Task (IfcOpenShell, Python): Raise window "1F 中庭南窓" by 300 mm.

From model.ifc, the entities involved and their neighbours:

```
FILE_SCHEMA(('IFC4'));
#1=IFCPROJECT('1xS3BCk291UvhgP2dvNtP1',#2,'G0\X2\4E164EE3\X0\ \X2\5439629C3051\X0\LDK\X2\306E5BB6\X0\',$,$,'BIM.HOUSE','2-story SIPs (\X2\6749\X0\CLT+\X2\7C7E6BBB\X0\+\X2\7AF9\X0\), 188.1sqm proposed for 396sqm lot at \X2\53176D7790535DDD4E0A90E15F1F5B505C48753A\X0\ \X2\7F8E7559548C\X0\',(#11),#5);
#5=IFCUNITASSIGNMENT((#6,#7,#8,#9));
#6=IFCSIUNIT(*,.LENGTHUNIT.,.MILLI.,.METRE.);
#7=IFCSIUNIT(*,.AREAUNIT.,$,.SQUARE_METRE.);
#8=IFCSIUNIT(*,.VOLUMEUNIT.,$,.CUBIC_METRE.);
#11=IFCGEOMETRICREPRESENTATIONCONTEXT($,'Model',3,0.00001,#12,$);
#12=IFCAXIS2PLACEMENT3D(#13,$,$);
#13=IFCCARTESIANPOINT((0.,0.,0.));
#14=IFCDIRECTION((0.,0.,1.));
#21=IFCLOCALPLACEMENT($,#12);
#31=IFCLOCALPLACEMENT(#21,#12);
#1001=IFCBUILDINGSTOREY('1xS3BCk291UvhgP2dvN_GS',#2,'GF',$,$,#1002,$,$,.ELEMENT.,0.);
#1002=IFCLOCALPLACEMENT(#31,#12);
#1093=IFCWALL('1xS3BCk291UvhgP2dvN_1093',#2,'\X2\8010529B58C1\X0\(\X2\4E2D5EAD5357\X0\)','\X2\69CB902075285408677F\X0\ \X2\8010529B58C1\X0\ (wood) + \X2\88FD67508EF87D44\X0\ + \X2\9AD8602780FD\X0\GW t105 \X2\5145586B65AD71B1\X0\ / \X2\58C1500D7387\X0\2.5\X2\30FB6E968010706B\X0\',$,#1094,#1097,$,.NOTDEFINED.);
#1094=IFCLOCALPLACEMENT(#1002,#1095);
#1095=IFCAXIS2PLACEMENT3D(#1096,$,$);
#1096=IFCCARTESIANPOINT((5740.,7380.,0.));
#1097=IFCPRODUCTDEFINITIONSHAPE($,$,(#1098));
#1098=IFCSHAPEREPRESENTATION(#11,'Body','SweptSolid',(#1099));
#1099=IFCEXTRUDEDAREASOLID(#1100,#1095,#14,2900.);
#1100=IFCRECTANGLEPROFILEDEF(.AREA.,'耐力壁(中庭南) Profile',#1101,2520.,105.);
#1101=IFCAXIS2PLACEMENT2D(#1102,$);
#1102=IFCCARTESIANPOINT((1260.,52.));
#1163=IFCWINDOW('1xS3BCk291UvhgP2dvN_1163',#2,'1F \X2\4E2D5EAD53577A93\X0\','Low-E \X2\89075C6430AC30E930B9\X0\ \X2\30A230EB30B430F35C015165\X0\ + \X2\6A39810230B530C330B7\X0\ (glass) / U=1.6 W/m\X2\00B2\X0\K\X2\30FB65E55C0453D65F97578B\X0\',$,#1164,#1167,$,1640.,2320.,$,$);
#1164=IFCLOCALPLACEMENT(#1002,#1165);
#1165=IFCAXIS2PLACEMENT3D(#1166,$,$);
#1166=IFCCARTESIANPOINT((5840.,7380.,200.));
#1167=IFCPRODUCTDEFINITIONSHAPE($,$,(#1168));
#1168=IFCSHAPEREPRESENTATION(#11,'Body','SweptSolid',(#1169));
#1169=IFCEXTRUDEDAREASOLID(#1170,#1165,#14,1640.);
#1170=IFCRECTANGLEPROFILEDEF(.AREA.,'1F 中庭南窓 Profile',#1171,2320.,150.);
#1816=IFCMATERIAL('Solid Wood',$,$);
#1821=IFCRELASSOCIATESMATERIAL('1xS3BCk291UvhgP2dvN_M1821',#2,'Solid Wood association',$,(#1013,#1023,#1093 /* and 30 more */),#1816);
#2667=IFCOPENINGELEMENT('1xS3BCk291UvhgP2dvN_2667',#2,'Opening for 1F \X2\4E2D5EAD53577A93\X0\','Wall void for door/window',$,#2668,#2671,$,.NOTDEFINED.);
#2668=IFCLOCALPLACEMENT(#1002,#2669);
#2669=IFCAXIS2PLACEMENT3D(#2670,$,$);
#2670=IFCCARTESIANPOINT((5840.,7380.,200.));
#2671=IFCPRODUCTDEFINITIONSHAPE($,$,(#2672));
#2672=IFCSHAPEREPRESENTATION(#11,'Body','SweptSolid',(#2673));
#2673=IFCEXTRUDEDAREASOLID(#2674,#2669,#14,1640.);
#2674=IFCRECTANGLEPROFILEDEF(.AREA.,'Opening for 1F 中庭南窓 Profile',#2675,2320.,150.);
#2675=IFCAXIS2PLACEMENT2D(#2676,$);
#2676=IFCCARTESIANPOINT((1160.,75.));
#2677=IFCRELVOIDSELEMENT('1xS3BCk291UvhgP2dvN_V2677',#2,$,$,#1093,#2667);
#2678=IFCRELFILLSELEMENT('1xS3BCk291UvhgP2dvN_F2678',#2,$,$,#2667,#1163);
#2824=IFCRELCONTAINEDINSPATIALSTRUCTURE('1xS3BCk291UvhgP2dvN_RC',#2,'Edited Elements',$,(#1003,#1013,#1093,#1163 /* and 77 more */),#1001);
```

```python
import numpy as np
import ifcopenshell
import ifcopenshell.api.geometry
import ifcopenshell.util.placement
import ifcopenshell.util.unit

model = ifcopenshell.open("model.ifc")
unit_scale = ifcopenshell.util.unit.calculate_unit_scale(model)

window = model.by_guid("1xS3BCk291UvhgP2dvN_1163")
opening = window.FillsVoids[0].RelatingOpeningElement
dz = 0.3 / unit_scale

shift = np.array([0.0, 0.0, dz])
# The window is not placed relative to its opening, so move both.
for product in (opening, window):
    matrix = ifcopenshell.util.placement.get_local_placement(product.ObjectPlacement)
    matrix[:3, 3] += shift
    ifcopenshell.api.geometry.edit_object_placement(model, product=product, matrix=matrix, is_si=False)

print(f"moved by {dz * unit_scale:+.3f} m")

model.write("model_rev.ifc")
```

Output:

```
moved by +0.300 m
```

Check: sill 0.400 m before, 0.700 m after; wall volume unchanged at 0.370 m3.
